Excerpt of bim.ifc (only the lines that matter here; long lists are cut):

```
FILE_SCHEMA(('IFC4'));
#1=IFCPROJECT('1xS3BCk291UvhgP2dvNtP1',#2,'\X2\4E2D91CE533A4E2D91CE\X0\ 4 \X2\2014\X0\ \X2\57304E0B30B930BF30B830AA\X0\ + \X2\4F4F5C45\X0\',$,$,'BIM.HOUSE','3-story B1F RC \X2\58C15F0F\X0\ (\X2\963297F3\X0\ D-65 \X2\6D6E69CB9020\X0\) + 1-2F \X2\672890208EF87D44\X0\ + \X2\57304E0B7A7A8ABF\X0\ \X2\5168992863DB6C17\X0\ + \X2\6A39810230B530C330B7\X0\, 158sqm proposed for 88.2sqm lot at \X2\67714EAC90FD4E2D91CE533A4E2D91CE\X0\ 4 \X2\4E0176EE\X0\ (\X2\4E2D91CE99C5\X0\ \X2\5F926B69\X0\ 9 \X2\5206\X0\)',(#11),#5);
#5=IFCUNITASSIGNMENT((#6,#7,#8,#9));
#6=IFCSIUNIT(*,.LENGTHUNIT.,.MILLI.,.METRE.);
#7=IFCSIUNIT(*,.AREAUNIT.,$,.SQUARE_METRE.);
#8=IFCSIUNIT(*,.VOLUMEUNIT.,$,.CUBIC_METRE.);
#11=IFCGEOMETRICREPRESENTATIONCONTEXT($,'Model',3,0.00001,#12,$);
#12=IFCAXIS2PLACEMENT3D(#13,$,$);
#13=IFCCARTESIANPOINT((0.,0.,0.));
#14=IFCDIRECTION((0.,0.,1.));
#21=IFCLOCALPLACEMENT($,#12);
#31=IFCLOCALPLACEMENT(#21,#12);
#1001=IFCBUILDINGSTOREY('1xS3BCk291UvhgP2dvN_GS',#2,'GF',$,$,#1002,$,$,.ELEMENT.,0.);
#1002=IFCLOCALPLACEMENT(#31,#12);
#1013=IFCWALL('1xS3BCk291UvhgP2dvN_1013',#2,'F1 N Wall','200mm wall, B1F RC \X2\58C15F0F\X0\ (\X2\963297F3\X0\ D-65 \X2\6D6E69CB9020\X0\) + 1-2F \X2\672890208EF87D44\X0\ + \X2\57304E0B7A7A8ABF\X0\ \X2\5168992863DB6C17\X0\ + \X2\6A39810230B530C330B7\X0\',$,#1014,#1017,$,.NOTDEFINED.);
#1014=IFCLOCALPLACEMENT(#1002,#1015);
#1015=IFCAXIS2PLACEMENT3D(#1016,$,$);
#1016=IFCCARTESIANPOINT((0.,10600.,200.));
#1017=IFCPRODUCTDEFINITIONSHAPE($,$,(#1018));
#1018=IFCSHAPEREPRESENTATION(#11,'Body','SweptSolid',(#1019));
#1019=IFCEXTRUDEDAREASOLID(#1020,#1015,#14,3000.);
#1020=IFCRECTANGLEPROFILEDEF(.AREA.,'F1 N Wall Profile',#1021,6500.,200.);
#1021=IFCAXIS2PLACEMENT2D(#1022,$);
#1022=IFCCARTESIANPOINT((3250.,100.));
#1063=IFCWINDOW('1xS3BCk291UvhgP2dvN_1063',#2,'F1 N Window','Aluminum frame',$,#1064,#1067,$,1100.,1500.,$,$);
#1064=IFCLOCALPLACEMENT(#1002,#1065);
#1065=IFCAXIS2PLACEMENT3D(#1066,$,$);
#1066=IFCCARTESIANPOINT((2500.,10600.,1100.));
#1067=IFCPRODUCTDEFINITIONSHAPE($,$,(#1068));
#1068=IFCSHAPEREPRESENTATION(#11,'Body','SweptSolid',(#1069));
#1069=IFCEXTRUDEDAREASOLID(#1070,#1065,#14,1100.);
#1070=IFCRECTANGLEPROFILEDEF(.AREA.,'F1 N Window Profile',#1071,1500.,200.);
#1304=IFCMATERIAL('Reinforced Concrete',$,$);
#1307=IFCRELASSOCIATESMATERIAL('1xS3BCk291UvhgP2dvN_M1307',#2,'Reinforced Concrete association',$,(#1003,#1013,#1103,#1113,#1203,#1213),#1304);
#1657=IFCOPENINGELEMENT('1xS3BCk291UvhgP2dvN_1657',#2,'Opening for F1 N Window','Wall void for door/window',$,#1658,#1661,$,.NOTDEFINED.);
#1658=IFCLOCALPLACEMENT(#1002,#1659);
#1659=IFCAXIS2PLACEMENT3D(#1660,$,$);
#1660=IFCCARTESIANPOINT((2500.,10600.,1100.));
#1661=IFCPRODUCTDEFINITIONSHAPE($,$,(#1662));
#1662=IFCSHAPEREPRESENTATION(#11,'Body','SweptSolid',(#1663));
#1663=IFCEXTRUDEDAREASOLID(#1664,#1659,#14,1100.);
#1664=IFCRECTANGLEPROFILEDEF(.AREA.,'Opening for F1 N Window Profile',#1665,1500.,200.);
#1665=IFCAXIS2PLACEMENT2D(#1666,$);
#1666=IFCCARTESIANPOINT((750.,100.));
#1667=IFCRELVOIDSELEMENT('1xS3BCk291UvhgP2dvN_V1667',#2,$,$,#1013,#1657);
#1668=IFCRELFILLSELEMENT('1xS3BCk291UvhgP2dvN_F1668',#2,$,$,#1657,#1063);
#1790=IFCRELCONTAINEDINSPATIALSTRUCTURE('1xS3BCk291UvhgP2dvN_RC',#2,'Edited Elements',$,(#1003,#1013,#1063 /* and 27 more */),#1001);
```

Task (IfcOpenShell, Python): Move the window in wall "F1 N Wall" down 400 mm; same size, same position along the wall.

```python
import numpy as np
import ifcopenshell
import ifcopenshell.api.geometry
import ifcopenshell.util.placement
import ifcopenshell.util.unit

model = ifcopenshell.open("bim.ifc")
unit_scale = ifcopenshell.util.unit.calculate_unit_scale(model)

window = model.by_guid("1xS3BCk291UvhgP2dvN_1063")
opening = window.FillsVoids[0].RelatingOpeningElement
dz = -0.4 / unit_scale

shift = np.array([0.0, 0.0, dz])
# The window is not placed relative to its opening, so move both.
for product in (opening, window):
    matrix = ifcopenshell.util.placement.get_local_placement(product.ObjectPlacement)
    matrix[:3, 3] += shift
    ifcopenshell.api.geometry.edit_object_placement(model, product=product, matrix=matrix, is_si=False)

print(f"moved by {dz * unit_scale:+.3f} m")

model.write("bim-out.ifc")
```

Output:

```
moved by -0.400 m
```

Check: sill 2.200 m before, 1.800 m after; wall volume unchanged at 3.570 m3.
